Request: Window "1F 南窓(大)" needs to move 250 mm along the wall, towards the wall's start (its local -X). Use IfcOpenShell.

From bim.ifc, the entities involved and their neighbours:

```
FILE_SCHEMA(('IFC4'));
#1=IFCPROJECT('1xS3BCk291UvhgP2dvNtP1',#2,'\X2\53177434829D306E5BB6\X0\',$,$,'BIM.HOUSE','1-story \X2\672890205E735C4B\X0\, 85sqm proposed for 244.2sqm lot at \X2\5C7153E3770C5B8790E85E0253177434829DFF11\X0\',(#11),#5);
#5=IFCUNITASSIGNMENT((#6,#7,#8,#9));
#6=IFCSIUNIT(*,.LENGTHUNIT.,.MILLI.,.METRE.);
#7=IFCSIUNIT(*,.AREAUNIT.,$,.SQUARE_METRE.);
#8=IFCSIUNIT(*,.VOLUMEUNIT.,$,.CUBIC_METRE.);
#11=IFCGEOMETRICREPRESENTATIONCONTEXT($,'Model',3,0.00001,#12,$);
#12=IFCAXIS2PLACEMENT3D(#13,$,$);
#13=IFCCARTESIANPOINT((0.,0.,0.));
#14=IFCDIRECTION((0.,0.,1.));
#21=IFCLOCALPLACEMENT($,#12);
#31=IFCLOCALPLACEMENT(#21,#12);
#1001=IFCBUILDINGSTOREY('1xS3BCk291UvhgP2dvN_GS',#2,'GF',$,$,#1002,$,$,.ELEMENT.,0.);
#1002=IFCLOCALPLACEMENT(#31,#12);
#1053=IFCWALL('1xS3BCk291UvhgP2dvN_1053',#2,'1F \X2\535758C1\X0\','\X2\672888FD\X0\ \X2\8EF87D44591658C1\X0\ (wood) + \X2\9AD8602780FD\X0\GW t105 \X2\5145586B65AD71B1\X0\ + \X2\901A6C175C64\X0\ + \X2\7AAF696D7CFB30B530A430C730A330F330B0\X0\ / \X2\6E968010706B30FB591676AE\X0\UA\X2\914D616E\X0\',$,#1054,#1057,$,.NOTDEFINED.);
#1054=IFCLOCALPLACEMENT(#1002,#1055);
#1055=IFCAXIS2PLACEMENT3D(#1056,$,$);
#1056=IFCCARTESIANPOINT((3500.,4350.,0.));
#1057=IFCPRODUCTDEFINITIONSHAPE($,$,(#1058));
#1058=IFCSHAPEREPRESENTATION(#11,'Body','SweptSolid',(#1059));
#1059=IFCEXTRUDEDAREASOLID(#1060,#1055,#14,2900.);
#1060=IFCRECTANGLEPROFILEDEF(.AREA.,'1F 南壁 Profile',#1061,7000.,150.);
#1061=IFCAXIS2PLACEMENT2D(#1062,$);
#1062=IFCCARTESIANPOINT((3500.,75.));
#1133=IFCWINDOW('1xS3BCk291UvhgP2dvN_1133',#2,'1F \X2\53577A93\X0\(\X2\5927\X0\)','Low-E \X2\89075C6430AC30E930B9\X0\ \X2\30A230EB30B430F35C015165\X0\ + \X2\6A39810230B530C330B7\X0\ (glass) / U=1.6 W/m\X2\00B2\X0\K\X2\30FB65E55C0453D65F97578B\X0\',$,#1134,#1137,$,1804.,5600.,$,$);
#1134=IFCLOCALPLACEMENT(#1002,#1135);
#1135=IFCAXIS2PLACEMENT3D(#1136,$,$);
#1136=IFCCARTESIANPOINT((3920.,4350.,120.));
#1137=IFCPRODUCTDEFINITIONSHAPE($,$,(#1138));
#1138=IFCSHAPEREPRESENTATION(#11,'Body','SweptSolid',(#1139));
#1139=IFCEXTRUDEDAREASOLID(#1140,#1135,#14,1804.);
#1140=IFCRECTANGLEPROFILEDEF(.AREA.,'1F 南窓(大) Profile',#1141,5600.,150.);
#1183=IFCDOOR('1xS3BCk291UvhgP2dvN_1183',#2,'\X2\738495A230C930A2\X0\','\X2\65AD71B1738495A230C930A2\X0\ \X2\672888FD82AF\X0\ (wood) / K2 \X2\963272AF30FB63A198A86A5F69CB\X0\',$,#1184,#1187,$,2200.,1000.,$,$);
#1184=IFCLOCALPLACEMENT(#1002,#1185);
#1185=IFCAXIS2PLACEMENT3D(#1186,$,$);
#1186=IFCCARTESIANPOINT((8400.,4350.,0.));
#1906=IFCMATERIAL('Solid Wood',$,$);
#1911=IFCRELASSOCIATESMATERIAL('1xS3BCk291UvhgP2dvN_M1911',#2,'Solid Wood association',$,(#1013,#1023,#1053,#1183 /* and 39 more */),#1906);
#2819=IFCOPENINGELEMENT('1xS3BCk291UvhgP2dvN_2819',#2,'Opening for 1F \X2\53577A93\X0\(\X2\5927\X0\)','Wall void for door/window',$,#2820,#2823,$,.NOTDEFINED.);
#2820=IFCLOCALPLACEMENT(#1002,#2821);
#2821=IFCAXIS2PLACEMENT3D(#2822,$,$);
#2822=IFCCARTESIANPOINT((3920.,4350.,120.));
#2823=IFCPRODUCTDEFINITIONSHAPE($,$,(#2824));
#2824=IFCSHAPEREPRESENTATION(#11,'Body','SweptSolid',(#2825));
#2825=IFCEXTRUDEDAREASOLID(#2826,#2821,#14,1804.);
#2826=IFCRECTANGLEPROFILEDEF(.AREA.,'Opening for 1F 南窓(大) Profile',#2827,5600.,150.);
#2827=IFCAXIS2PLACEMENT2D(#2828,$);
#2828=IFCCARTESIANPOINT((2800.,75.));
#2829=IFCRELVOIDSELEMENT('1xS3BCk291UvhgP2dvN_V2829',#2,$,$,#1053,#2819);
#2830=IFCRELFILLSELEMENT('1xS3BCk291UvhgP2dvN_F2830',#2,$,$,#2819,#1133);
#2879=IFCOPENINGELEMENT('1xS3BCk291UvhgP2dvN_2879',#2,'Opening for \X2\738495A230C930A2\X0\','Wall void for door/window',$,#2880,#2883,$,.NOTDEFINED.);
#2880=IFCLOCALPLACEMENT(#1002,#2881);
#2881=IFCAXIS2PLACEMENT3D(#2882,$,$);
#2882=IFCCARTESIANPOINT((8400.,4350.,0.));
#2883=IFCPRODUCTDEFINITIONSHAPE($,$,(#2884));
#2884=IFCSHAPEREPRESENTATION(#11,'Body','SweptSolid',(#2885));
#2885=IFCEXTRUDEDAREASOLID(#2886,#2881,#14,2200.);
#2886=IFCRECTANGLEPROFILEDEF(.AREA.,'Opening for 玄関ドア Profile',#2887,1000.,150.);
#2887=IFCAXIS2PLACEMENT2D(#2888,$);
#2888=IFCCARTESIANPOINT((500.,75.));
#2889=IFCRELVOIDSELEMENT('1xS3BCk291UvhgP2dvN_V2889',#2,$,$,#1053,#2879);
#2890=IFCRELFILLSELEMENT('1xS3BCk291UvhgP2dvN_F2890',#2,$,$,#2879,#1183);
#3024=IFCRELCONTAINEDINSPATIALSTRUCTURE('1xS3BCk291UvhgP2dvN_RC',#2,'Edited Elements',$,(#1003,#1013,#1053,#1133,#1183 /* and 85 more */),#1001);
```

```python
import ifcopenshell
import ifcopenshell.api.geometry
import ifcopenshell.util.placement

model = ifcopenshell.open("bim.ifc")

window = model.by_guid("1xS3BCk291UvhgP2dvN_1133")
opening = window.FillsVoids[0].RelatingOpeningElement
wall = opening.VoidsElements[0].RelatingBuildingElement

wall_matrix = ifcopenshell.util.placement.get_local_placement(wall.ObjectPlacement)
shift = wall_matrix[:3, 0] * -250.0
before = ifcopenshell.util.placement.get_local_placement(window.ObjectPlacement)[:3, 3].copy()

# The window is not placed relative to its opening, so move both.
for product in (opening, window):
    matrix = ifcopenshell.util.placement.get_local_placement(product.ObjectPlacement)
    matrix[:3, 3] += shift
    ifcopenshell.api.geometry.edit_object_placement(model, product=product, matrix=matrix, is_si=False)

after = ifcopenshell.util.placement.get_local_placement(window.ObjectPlacement)[:3, 3]
print("window moved by", (after - before).round(3) + 0.0)

model.write("bim_v2.ifc")
```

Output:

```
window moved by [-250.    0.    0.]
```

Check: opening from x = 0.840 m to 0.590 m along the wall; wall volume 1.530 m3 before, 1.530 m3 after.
